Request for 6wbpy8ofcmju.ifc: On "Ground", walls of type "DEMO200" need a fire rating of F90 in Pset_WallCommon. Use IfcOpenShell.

First a look at what the model holds.

```python
import ifcopenshell
import ifcopenshell.util.element

model = ifcopenshell.open("6wbpy8ofcmju.ifc")
print(model.schema)
storey = next(s for s in model.by_type("IfcBuildingStorey") if s.Name == "Ground")
walls = [e for e in ifcopenshell.util.element.get_decomposition(storey) if e.is_a("IfcWall")]
seen = {}
for e in walls:
    element_type = ifcopenshell.util.element.get_type(e)
    key = (element_type.Name if element_type != e and element_type else None, ifcopenshell.util.element.get_pset(e, "Pset_WallCommon", "FireRating"))
    seen[key] = seen.get(key, 0) + 1
for (name, value), count in sorted(seen.items(), key=str):
    print(count, "x", name, "|", value)
```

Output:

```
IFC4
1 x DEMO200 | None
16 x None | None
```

```python
import ifcopenshell
import ifcopenshell.api.pset
import ifcopenshell.util.element

model = ifcopenshell.open("6wbpy8ofcmju.ifc")

storey = next(s for s in model.by_type("IfcBuildingStorey") if s.Name == "Ground")
walls = [e for e in ifcopenshell.util.element.get_decomposition(storey) if e.is_a("IfcWall")]

count = 0
for e in walls:
    element_type = ifcopenshell.util.element.get_type(e)
    if element_type in (None, e) or element_type.Name != "DEMO200":
        continue
    # add_pset returns the element's existing set when there is one.
    pset = ifcopenshell.api.pset.add_pset(model, product=e, name="Pset_WallCommon")
    ifcopenshell.api.pset.edit_pset(model, pset=pset, properties={"FireRating": "F90"})
    count += 1

print(count, "walls updated")

model.write("6wbpy8ofcmju_updated.ifc")
```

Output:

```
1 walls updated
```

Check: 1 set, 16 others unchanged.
